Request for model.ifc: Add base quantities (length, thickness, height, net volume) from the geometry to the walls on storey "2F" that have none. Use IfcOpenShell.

First a look at what the model holds.

```python
import ifcopenshell
import ifcopenshell.util.element
import ifcopenshell.util.unit

model = ifcopenshell.open("model.ifc")
print(model.schema)
for unit_type in ("LENGTHUNIT", "AREAUNIT", "VOLUMEUNIT"):
    print(unit_type, ifcopenshell.util.unit.calculate_unit_scale(model, unit_type))
storey = next(s for s in model.by_type("IfcBuildingStorey") if s.Name == "2F")
walls = [e for e in ifcopenshell.util.element.get_decomposition(storey) if e.is_a("IfcWall")]
for e in sorted(walls, key=lambda e: e.id()):
    print(e.id(), e.is_a(), e.Name, list(ifcopenshell.util.element.get_psets(e, qtos_only=True)), sep=" | ")
```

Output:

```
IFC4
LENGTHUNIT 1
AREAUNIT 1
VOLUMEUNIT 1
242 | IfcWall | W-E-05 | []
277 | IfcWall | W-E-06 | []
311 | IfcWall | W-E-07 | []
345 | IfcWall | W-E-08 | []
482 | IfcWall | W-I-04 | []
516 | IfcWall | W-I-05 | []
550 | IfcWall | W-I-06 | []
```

```python
import ifcopenshell
import ifcopenshell.api.pset
import ifcopenshell.geom
import ifcopenshell.util.element
import ifcopenshell.util.shape
import ifcopenshell.util.unit

model = ifcopenshell.open("model.ifc")
unit_scale = ifcopenshell.util.unit.calculate_unit_scale(model)
volume_scale = ifcopenshell.util.unit.calculate_unit_scale(model, "VOLUMEUNIT")
settings = ifcopenshell.geom.settings()

storey = next(s for s in model.by_type("IfcBuildingStorey") if s.Name == "2F")
walls = [e for e in ifcopenshell.util.element.get_decomposition(storey) if e.is_a("IfcWall")]

for e in sorted(walls, key=lambda e: e.id()):
    if ifcopenshell.util.element.get_psets(e, qtos_only=True, should_inherit=False):
        continue
    # Geometry comes back in metres, in the element's own axes.
    shape = ifcopenshell.geom.create_shape(settings, e)
    values = {
        "Length": ifcopenshell.util.shape.get_x(shape.geometry) / unit_scale,
        "Width": ifcopenshell.util.shape.get_y(shape.geometry) / unit_scale,
        "Height": ifcopenshell.util.shape.get_z(shape.geometry) / unit_scale,
        "NetVolume": ifcopenshell.util.shape.get_volume(shape.geometry) / volume_scale,
    }
    qto = ifcopenshell.api.pset.add_qto(model, product=e, name="Qto_WallBaseQuantities")
    ifcopenshell.api.pset.edit_qto(model, qto=qto, properties=values)
    print(e.id(), {k: round(v, 3) for k, v in values.items()})

model.write("model_updated.ifc")
```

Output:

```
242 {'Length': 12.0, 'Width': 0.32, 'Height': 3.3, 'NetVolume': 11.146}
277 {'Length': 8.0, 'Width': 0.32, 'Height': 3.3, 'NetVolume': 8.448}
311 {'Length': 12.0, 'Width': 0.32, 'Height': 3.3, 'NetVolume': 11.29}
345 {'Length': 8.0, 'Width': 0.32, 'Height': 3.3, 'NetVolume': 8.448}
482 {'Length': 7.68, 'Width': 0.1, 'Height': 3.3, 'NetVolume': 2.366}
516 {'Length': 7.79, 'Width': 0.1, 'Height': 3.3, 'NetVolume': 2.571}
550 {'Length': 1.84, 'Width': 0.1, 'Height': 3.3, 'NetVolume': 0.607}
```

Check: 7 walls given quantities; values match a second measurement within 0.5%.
